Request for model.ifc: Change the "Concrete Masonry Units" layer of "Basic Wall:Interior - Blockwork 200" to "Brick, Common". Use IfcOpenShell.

First a look at what the model holds.

```python
import ifcopenshell
import ifcopenshell.util.element

model = ifcopenshell.open("model.ifc")
print(model.schema)
for layer_set in model.by_type("IfcMaterialLayerSet"):
    if layer_set.LayerSetName == "Basic Wall:Interior - Blockwork 200":
        for layer in layer_set.MaterialLayers:
            print(layer.id(), layer.Material and layer.Material.Name, layer.LayerThickness, sep=" | ")
        print(len(ifcopenshell.util.element.get_elements_by_material(model, layer_set)), "elements and types use it")
print(sorted(m.Name for m in model.by_type("IfcMaterial") if m.Name)[:60])
```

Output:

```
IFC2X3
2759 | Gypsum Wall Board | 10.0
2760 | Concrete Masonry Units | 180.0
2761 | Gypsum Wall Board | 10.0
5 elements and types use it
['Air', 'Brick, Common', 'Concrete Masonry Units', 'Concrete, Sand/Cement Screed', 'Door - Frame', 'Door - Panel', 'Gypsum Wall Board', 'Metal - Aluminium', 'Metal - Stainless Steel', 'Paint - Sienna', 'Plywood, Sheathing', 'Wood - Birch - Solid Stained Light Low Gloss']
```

```python
import ifcopenshell
import ifcopenshell.api.material

model = ifcopenshell.open("model.ifc")

layer_set = next(s for s in model.by_type("IfcMaterialLayerSet") if s.LayerSetName == "Basic Wall:Interior - Blockwork 200")
layer = next(l for l in layer_set.MaterialLayers if l.Material and l.Material.Name == "Concrete Masonry Units")
material = next(m for m in model.by_type("IfcMaterial") if m.Name == "Brick, Common")

# Point this one layer at the other material; renaming the old one would change it everywhere.
ifcopenshell.api.material.edit_layer(model, layer=layer, attributes={}, material=material)

print([l.Material.Name if l.Material else None for l in layer_set.MaterialLayers])

model.write("model-out.ifc")
```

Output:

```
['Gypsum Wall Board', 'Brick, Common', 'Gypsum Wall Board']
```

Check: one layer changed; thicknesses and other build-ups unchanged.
